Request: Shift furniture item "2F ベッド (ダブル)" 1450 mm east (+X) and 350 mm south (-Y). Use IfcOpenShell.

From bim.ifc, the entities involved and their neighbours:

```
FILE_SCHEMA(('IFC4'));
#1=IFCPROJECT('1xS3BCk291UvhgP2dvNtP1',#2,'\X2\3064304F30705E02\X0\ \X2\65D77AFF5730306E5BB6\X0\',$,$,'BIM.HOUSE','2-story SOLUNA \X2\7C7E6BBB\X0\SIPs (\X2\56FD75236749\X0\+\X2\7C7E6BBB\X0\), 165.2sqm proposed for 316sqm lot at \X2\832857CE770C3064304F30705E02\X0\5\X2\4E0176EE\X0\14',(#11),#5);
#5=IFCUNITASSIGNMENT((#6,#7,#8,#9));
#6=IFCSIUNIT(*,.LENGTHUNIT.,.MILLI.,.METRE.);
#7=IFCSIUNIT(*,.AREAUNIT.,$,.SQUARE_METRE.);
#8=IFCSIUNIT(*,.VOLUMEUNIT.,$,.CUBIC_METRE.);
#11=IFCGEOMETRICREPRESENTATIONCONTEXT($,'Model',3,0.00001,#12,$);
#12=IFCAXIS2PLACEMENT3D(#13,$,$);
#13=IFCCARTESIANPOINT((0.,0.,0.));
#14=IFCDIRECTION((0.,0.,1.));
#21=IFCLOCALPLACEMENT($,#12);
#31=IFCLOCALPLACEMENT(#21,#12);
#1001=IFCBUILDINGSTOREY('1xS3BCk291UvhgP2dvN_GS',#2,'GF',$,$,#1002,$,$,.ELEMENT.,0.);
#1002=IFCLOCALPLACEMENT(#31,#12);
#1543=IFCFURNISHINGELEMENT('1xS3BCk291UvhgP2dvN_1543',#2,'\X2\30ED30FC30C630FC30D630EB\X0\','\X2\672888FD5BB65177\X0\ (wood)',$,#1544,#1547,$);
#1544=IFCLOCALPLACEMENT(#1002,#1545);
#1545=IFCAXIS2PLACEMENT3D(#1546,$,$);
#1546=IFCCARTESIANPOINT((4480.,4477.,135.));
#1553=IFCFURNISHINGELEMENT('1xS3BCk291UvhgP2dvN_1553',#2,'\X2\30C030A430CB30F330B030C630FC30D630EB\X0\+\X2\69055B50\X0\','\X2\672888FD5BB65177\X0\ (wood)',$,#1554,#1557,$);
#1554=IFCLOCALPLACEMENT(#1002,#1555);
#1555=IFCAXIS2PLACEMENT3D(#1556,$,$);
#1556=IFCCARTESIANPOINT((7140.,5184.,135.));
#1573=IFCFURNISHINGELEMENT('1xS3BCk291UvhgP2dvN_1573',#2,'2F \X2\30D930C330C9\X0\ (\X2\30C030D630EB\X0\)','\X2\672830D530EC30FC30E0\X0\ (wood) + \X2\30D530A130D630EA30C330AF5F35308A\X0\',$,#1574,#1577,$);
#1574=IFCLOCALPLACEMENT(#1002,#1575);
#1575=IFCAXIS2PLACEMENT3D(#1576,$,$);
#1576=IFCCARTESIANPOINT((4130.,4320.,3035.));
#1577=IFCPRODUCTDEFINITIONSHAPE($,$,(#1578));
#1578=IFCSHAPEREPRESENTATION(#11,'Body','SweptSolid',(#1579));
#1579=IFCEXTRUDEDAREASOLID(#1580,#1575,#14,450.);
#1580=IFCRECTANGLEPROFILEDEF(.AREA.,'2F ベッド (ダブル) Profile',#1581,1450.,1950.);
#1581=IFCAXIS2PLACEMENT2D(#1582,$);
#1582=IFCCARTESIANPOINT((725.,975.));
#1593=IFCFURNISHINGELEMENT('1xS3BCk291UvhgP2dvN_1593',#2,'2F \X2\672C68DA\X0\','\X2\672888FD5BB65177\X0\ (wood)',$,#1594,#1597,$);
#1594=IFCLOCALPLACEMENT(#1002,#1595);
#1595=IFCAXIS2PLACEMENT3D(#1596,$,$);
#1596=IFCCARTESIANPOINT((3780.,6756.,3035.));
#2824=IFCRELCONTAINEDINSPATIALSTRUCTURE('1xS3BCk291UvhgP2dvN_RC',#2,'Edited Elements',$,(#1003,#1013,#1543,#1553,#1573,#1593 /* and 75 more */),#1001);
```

```python
import ifcopenshell
import ifcopenshell.api.geometry
import ifcopenshell.util.placement
import ifcopenshell.util.unit

model = ifcopenshell.open("bim.ifc")
unit_scale = ifcopenshell.util.unit.calculate_unit_scale(model)

item = model.by_guid("1xS3BCk291UvhgP2dvN_1573")
matrix = ifcopenshell.util.placement.get_local_placement(item.ObjectPlacement)
matrix[0, 3] += 1.45 / unit_scale
matrix[1, 3] -= 0.35 / unit_scale
ifcopenshell.api.geometry.edit_object_placement(model, product=item, matrix=matrix, is_si=False)

print(ifcopenshell.util.placement.get_local_placement(item.ObjectPlacement).round(3) + 0.0)

model.write("bim_v2.ifc")
```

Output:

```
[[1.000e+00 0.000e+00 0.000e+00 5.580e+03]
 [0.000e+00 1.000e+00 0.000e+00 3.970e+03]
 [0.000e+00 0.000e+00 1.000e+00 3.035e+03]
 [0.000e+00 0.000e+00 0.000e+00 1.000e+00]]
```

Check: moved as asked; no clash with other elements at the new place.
